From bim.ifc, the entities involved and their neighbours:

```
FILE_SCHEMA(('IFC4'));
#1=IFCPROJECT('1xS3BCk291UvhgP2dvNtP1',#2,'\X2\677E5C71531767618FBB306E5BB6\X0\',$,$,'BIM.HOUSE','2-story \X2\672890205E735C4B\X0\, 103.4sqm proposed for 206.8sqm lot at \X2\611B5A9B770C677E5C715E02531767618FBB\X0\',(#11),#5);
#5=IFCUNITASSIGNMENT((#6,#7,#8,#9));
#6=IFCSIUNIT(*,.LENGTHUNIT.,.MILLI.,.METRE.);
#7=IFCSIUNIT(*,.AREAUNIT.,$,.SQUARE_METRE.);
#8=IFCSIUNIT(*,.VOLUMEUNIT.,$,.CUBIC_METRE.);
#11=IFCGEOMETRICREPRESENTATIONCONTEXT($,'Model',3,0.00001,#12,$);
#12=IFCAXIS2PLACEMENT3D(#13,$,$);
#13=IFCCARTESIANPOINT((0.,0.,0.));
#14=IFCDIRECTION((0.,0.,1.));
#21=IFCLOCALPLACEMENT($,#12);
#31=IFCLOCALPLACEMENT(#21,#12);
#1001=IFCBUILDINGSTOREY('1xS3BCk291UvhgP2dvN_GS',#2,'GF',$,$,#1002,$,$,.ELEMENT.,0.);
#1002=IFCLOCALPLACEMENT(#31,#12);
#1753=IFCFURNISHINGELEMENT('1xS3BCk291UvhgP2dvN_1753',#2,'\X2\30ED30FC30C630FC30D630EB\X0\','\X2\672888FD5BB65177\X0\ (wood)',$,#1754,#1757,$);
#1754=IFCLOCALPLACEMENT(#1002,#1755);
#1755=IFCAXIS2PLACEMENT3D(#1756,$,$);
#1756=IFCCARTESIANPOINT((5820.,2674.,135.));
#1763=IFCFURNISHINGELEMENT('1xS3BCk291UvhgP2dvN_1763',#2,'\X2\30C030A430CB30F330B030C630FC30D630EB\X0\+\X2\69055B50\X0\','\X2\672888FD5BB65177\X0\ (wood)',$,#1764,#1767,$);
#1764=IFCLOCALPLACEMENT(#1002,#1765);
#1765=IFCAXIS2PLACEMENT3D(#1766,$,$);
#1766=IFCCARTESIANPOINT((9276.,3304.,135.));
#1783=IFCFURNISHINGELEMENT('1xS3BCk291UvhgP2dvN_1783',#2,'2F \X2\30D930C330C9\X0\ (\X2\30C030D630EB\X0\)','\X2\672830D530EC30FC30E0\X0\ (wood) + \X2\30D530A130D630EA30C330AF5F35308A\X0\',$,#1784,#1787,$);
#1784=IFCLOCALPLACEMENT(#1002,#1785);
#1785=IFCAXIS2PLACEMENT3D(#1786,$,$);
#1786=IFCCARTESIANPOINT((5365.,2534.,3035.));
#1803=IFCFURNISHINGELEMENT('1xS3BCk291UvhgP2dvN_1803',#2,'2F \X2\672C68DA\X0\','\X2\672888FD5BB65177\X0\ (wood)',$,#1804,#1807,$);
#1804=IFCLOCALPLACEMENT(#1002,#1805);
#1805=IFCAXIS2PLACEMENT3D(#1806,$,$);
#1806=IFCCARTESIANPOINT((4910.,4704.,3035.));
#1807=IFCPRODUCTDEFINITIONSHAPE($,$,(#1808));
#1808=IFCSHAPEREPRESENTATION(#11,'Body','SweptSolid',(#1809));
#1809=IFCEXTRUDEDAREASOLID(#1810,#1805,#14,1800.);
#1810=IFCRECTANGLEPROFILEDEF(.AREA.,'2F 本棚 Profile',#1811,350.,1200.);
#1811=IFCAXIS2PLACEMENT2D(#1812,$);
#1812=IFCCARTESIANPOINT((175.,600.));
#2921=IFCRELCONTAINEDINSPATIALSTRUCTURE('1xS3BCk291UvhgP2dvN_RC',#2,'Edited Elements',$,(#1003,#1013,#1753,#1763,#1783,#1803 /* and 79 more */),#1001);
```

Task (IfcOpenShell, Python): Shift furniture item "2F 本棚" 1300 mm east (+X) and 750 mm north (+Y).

```python
import ifcopenshell
import ifcopenshell.api.geometry
import ifcopenshell.util.placement
import ifcopenshell.util.unit

model = ifcopenshell.open("bim.ifc")
unit_scale = ifcopenshell.util.unit.calculate_unit_scale(model)

item = model.by_id(1803)
matrix = ifcopenshell.util.placement.get_local_placement(item.ObjectPlacement)
matrix[0, 3] += 1.3 / unit_scale
matrix[1, 3] += 0.75 / unit_scale
ifcopenshell.api.geometry.edit_object_placement(model, product=item, matrix=matrix, is_si=False)

print(ifcopenshell.util.placement.get_local_placement(item.ObjectPlacement).round(3) + 0.0)

model.write("bim-out.ifc")
```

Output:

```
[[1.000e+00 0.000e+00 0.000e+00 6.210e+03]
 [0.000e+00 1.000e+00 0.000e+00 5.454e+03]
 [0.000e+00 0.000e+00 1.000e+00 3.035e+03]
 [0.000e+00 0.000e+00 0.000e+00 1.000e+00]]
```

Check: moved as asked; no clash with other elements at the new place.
